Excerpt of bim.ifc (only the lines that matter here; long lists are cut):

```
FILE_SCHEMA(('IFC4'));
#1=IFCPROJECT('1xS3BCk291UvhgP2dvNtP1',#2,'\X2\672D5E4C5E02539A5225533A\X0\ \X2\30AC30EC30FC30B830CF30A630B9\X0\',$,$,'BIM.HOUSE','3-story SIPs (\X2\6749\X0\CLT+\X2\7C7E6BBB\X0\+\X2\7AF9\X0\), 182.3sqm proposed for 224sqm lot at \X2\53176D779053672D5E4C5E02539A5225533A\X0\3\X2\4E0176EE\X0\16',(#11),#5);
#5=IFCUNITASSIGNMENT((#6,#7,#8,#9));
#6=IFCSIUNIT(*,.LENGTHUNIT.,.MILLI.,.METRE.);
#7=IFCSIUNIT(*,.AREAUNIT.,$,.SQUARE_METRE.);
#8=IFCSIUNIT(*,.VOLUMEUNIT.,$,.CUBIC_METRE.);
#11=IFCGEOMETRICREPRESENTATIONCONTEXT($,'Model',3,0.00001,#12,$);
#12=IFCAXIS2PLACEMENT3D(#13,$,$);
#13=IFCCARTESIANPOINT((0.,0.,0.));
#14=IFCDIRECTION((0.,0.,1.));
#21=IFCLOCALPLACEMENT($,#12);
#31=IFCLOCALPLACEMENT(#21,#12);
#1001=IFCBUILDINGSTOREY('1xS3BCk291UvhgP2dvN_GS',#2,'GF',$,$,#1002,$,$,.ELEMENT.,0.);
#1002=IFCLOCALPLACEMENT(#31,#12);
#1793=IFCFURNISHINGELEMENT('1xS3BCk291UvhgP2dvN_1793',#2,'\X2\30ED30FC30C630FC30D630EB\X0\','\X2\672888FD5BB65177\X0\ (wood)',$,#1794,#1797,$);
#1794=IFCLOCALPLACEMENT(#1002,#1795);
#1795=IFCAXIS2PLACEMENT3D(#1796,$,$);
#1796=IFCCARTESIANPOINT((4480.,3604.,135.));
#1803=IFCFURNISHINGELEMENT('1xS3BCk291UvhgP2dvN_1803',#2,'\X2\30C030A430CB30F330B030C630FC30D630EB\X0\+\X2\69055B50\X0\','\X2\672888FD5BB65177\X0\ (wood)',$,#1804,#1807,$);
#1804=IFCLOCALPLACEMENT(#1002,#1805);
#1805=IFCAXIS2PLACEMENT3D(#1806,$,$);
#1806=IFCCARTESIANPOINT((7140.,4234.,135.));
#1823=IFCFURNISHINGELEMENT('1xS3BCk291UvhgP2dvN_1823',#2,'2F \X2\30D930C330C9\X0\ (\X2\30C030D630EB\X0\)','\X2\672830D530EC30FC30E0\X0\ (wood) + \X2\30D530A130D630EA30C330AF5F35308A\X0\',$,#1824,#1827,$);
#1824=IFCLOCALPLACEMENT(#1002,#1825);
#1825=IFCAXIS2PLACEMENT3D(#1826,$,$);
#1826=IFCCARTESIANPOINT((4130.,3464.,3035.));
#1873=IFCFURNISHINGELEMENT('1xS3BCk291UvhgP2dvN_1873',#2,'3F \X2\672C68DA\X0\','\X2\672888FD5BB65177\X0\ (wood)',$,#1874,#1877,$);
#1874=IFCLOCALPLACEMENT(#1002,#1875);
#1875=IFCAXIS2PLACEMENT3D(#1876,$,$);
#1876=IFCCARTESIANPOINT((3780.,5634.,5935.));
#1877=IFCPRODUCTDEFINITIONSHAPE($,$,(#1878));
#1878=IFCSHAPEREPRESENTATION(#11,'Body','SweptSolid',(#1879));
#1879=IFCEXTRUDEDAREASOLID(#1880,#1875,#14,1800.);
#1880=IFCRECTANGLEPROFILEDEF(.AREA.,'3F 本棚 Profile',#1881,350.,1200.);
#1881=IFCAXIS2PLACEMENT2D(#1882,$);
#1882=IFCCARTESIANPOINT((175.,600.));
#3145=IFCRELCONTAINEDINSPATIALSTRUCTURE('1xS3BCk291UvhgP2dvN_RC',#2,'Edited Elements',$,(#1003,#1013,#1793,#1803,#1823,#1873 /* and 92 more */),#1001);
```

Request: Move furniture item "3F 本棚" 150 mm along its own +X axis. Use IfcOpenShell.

```python
import ifcopenshell
import ifcopenshell.api.geometry
import ifcopenshell.util.placement
import ifcopenshell.util.unit

model = ifcopenshell.open("bim.ifc")
unit_scale = ifcopenshell.util.unit.calculate_unit_scale(model)

item = model.by_guid("1xS3BCk291UvhgP2dvN_1873")
matrix = ifcopenshell.util.placement.get_local_placement(item.ObjectPlacement)
matrix[:3, 3] += matrix[:3, 0] * 0.15 / unit_scale
ifcopenshell.api.geometry.edit_object_placement(model, product=item, matrix=matrix, is_si=False)

print(ifcopenshell.util.placement.get_local_placement(item.ObjectPlacement).round(3) + 0.0)

model.write("bim_edited.ifc")
```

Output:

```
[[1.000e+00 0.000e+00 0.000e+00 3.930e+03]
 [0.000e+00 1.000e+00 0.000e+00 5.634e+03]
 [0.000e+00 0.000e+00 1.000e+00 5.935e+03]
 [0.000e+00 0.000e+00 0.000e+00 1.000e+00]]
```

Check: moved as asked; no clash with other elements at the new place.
